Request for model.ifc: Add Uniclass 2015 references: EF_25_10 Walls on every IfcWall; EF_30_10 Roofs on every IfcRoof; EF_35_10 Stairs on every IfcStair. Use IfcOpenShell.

First a look at what the model holds.

```python
import ifcopenshell

model = ifcopenshell.open("model.ifc")
print(model.schema)
print("classifications:", [c.Name for c in model.by_type("IfcClassification")])
for ifc_class in ("IfcDoor", "IfcRoof", "IfcStair", "IfcWall", "IfcWindow"):
    print(ifc_class, len(model.by_type(ifc_class)))
```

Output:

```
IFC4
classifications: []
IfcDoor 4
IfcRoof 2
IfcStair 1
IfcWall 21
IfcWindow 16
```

```python
import ifcopenshell
import ifcopenshell.api.classification

model = ifcopenshell.open("model.ifc")

system = ifcopenshell.api.classification.add_classification(model, classification="Uniclass 2015")

codes = {
    "IfcWall": ("EF_25_10", "Walls"),
    "IfcRoof": ("EF_30_10", "Roofs"),
    "IfcStair": ("EF_35_10", "Stairs"),
}
for ifc_class, (code, name) in codes.items():
    products = model.by_type(ifc_class)
    ifcopenshell.api.classification.add_reference(
        model, products=products, classification=system, identification=code, name=name
    )
    print(code, len(products))

model.write("model_rev.ifc")
```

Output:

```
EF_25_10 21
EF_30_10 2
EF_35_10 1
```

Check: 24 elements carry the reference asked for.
